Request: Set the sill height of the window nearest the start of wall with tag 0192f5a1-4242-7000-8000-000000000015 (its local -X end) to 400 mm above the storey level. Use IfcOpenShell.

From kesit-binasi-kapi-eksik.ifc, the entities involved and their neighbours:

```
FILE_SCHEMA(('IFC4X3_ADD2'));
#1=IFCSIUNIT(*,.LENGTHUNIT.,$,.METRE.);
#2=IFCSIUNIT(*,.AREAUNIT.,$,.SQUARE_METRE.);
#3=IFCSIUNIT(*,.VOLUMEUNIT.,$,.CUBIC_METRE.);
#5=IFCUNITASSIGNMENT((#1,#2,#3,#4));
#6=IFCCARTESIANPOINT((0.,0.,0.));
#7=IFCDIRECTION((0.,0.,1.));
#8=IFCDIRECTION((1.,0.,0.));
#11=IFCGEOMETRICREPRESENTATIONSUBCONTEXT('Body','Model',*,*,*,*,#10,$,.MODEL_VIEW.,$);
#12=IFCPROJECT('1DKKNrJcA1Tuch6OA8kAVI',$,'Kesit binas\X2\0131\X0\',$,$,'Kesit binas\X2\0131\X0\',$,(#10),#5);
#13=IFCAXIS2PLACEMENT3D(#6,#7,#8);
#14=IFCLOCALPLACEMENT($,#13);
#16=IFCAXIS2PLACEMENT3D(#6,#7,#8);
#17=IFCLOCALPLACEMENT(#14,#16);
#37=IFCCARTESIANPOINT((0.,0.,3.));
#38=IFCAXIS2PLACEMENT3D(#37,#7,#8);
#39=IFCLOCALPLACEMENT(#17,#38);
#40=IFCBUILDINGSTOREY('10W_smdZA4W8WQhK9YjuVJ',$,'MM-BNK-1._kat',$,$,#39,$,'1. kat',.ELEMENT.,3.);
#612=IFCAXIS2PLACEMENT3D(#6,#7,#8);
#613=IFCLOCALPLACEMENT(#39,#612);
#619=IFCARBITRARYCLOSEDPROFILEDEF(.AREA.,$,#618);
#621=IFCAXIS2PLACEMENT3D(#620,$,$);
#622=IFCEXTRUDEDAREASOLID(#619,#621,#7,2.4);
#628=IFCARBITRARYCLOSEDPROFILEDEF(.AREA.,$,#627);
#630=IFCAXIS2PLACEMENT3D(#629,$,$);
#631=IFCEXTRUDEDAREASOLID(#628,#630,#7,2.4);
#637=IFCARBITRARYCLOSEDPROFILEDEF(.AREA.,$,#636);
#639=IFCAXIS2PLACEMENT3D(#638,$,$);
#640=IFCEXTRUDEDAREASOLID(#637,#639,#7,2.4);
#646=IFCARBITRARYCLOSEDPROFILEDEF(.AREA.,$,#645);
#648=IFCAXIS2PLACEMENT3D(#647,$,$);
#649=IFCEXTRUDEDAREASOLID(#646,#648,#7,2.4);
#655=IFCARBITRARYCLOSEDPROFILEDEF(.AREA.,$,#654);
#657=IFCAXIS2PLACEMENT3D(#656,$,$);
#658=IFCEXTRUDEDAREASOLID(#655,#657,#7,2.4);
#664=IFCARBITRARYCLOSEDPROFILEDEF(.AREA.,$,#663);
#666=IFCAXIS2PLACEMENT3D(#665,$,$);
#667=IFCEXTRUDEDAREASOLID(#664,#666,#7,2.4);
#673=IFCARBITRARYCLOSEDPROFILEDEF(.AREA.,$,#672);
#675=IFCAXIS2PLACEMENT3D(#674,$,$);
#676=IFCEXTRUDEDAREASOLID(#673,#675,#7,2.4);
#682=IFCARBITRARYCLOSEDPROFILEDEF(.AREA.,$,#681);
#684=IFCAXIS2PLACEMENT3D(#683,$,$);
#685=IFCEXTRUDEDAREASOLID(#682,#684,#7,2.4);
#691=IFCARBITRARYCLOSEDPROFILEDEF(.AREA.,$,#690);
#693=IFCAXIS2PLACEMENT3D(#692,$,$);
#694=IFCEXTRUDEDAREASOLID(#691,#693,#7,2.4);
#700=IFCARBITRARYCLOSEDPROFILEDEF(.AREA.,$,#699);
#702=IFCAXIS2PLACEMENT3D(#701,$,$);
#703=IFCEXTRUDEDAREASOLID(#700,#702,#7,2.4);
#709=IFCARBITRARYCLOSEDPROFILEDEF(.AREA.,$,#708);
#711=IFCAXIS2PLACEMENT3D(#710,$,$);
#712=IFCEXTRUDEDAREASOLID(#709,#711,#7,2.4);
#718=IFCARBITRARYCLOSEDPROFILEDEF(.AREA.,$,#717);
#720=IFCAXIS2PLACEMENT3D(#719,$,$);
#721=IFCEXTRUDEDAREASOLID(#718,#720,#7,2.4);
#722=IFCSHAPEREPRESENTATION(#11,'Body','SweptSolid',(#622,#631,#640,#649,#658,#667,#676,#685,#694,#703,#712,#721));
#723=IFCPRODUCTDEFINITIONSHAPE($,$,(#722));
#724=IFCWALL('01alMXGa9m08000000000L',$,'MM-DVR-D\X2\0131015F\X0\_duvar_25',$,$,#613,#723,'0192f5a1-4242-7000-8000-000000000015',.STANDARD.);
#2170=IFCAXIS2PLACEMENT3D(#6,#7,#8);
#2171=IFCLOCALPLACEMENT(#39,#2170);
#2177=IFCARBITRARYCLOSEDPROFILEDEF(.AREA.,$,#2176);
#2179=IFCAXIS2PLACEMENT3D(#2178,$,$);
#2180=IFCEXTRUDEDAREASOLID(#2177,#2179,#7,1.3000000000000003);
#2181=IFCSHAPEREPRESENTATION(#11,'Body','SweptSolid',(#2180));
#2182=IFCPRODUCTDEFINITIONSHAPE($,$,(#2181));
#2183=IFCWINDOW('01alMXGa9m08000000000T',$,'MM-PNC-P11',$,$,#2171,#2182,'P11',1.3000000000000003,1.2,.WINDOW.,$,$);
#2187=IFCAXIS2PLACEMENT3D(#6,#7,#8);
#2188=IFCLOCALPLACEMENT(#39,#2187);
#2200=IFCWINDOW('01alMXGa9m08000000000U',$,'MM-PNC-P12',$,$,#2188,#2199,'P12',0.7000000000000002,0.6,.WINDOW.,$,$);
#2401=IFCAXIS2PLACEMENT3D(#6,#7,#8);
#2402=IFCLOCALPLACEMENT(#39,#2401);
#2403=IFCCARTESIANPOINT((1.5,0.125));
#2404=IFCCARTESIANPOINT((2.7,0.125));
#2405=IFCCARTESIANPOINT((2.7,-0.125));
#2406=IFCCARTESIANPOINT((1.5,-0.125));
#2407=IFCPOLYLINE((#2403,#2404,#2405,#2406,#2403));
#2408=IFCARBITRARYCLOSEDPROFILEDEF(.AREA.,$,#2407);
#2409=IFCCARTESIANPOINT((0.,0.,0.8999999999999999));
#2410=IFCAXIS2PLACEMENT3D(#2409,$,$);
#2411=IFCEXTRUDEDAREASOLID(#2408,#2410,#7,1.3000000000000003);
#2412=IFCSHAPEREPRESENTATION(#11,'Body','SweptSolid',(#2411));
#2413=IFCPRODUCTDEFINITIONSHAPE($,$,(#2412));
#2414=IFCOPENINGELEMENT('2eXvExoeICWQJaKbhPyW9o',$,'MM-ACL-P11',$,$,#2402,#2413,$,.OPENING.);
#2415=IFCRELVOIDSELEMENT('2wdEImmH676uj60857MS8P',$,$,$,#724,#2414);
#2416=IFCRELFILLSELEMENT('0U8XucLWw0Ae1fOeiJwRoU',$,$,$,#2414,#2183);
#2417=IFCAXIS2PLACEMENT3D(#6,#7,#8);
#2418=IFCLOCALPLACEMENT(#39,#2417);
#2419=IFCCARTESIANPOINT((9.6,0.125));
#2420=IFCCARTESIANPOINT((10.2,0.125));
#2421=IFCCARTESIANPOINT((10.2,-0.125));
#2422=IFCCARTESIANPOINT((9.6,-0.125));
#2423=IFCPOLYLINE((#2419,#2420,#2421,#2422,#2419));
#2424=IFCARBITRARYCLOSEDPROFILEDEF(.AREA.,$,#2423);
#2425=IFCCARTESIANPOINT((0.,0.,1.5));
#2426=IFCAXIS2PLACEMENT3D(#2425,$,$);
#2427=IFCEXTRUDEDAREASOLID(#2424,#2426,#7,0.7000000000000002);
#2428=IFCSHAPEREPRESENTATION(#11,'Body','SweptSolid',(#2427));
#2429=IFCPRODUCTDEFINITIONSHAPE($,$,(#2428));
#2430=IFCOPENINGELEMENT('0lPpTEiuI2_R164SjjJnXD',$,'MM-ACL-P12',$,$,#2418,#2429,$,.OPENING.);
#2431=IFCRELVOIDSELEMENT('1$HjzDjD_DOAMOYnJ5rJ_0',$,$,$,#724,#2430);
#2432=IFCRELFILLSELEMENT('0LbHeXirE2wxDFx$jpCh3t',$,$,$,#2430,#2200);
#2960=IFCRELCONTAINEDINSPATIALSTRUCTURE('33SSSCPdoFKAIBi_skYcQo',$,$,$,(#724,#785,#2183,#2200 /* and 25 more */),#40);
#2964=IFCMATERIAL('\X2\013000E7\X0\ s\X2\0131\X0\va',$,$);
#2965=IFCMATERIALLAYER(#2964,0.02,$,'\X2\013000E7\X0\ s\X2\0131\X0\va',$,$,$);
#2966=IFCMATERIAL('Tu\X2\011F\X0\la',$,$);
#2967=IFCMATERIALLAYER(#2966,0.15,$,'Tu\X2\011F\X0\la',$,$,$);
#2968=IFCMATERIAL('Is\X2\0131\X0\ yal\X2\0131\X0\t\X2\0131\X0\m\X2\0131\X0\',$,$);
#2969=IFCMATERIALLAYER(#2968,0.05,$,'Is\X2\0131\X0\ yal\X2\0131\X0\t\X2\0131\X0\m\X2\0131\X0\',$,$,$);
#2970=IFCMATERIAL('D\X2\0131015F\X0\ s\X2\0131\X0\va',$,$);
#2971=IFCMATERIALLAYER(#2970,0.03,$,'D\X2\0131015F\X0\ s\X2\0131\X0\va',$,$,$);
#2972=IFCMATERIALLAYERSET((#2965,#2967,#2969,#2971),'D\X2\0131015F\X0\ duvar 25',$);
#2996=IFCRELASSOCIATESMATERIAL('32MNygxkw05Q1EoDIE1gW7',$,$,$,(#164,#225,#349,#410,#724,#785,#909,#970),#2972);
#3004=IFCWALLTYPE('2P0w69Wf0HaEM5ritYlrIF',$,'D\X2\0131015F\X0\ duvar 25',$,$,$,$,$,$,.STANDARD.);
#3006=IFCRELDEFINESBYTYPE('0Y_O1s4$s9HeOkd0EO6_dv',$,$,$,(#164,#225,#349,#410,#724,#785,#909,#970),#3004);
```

```python
import numpy as np
import ifcopenshell
import ifcopenshell.api.geometry
import ifcopenshell.geom
import ifcopenshell.util.element
import ifcopenshell.util.placement
import ifcopenshell.util.shape
import ifcopenshell.util.unit

model = ifcopenshell.open("kesit-binasi-kapi-eksik.ifc")
unit_scale = ifcopenshell.util.unit.calculate_unit_scale(model)

window = model.by_guid("01alMXGa9m08000000000T")
opening = window.FillsVoids[0].RelatingOpeningElement
storey = ifcopenshell.util.element.get_container(window, ifc_class="IfcBuildingStorey")
level = ifcopenshell.util.placement.get_local_placement(storey.ObjectPlacement)[2, 3]

# The opening's origin need not be at the sill, so measure its lowest point.
shape = ifcopenshell.geom.create_shape(ifcopenshell.geom.settings(), opening)
bottom = ifcopenshell.util.shape.get_shape_bottom_elevation(shape, shape.geometry) / unit_scale
dz = level + 0.4 - bottom

shift = np.array([0.0, 0.0, dz])
# The window is not placed relative to its opening, so move both.
for product in (opening, window):
    matrix = ifcopenshell.util.placement.get_local_placement(product.ObjectPlacement)
    matrix[:3, 3] += shift
    ifcopenshell.api.geometry.edit_object_placement(model, product=product, matrix=matrix, is_si=False)

print(f"moved by {dz * unit_scale:+.3f} m")

model.write("kesit-binasi-kapi-eksik-out.ifc")
```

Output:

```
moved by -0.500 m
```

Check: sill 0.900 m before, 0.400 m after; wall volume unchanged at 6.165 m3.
